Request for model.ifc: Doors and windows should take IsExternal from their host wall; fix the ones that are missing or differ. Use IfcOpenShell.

First a look at what the model holds.

```python
import ifcopenshell
import ifcopenshell.util.element

model = ifcopenshell.open("model.ifc")
print(model.schema)
seen = {}
for e in model.by_type("IfcDoor") + model.by_type("IfcWindow"):
    if not e.FillsVoids:
        continue
    host = e.FillsVoids[0].RelatingOpeningElement.VoidsElements[0].RelatingBuildingElement
    own = ifcopenshell.util.element.get_pset(e, f"Pset_{e.is_a()[3:].removesuffix('StandardCase')}Common", "IsExternal")
    wall = ifcopenshell.util.element.get_pset(host, "Pset_WallCommon", "IsExternal")
    seen[e.is_a(), own, wall] = seen.get((e.is_a(), own, wall), 0) + 1
for (cls, own, wall), count in sorted(seen.items(), key=str):
    print(count, cls, "IsExternal:", own, "| host wall:", wall)
```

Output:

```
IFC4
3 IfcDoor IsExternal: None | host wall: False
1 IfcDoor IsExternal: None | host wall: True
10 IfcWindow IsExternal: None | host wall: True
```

```python
import ifcopenshell
import ifcopenshell.api.pset
import ifcopenshell.util.element

model = ifcopenshell.open("model.ifc")

count = 0
for ifc_class, pset_name in (("IfcDoor", "Pset_DoorCommon"), ("IfcWindow", "Pset_WindowCommon")):
    for e in model.by_type(ifc_class):
        if not e.FillsVoids:
            continue
        host = e.FillsVoids[0].RelatingOpeningElement.VoidsElements[0].RelatingBuildingElement
        external = ifcopenshell.util.element.get_pset(host, "Pset_WallCommon", "IsExternal")
        if external is None or ifcopenshell.util.element.get_pset(e, pset_name, "IsExternal") == external:
            continue
        pset = ifcopenshell.api.pset.add_pset(model, product=e, name=pset_name)
        ifcopenshell.api.pset.edit_pset(model, pset=pset, properties={"IsExternal": external})
        count += 1

print(count, "updated")

model.write("model_edited.ifc")
```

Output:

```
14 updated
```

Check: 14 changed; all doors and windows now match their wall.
